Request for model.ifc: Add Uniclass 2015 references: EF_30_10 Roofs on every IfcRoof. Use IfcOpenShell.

First a look at what the model holds.

```python
import ifcopenshell

model = ifcopenshell.open("model.ifc")
print(model.schema)
print("classifications:", [c.Name for c in model.by_type("IfcClassification")])
for ifc_class in ("IfcDoor", "IfcRoof", "IfcStair", "IfcWall", "IfcWindow"):
    print(ifc_class, len(model.by_type(ifc_class)))
```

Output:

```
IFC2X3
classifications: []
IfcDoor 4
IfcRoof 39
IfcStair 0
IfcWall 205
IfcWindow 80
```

```python
import ifcopenshell
import ifcopenshell.api.classification

model = ifcopenshell.open("model.ifc")

# IFC2X3 requires Source and Edition and has no link from the project to the system.
system = model.create_entity("IfcClassification", Source="NBS", Edition="2015", Name="Uniclass 2015")

codes = {
    "IfcRoof": ("EF_30_10", "Roofs"),
}
for ifc_class, (code, name) in codes.items():
    products = model.by_type(ifc_class)
    ifcopenshell.api.classification.add_reference(
        model, products=products, classification=system, identification=code, name=name
    )
    print(code, len(products))

model.write("model_updated.ifc")
```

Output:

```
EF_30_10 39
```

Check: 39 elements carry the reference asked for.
